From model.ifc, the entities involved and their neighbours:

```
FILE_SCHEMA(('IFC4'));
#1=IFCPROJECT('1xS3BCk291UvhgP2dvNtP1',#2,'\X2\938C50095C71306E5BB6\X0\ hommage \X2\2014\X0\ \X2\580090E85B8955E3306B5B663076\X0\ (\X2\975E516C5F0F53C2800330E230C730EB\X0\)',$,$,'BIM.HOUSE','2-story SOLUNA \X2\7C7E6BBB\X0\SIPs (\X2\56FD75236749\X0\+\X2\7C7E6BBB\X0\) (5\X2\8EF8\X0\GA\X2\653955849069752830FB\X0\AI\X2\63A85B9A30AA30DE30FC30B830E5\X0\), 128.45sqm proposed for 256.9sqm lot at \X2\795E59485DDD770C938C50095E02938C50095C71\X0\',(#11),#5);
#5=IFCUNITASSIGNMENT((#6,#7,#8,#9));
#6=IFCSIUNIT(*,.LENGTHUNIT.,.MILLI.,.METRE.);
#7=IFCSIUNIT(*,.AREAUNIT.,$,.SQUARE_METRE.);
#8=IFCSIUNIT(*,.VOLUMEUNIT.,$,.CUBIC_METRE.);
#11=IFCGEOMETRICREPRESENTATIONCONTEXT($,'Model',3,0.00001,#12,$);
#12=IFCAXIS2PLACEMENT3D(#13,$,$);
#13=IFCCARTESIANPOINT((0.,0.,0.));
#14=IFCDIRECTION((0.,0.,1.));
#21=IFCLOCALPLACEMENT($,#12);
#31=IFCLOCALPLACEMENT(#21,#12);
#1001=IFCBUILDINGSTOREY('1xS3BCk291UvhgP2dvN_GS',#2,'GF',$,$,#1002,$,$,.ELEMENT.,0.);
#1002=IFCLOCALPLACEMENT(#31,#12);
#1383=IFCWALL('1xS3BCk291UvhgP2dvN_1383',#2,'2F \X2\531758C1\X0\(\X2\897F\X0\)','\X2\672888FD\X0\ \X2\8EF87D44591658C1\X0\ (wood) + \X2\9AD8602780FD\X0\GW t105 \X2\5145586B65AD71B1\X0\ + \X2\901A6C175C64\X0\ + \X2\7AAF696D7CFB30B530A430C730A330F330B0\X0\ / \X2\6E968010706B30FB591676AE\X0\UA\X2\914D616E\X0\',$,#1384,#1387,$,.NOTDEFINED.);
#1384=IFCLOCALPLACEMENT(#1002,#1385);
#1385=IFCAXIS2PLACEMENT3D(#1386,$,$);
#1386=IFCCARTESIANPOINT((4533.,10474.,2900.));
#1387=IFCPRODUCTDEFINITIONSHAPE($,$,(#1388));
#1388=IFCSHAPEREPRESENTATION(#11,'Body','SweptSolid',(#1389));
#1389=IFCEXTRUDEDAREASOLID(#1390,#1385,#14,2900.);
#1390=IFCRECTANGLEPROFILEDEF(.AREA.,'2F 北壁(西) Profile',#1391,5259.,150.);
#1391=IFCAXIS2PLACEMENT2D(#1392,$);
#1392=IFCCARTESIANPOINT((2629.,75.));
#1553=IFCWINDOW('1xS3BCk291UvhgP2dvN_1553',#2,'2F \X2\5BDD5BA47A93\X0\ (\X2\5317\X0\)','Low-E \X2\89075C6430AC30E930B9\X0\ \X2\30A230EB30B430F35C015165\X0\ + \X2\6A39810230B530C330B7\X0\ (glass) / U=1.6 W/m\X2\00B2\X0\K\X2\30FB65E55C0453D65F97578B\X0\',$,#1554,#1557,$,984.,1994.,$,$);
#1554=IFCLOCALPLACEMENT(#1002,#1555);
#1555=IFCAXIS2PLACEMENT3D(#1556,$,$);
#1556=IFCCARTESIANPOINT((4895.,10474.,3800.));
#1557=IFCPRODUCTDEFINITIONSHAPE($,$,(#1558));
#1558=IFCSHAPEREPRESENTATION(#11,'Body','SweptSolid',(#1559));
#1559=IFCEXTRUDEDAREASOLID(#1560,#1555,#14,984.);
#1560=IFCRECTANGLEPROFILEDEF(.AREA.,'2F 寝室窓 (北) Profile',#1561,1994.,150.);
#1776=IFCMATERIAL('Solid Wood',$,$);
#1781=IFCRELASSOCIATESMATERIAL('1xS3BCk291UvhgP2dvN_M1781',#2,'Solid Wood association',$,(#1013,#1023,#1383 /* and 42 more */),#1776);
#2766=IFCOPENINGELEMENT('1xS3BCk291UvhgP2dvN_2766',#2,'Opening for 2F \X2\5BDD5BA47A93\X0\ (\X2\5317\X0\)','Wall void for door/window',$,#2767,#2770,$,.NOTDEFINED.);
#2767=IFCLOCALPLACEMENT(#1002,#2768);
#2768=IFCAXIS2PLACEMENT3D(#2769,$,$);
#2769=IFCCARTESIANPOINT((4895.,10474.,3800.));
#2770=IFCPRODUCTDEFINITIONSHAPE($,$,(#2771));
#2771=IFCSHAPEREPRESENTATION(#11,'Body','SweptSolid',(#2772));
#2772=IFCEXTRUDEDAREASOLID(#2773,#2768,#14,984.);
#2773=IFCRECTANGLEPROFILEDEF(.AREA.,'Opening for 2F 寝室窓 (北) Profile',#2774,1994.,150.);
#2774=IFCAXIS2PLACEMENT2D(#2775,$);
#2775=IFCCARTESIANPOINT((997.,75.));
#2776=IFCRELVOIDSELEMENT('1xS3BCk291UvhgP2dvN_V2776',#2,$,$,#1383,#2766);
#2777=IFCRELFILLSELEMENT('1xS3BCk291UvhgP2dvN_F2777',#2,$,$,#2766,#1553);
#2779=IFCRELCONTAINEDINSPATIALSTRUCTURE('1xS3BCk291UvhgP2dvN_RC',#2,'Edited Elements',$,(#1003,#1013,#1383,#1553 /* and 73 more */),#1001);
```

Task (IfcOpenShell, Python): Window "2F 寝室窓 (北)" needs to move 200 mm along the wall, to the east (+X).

```python
import ifcopenshell
import ifcopenshell.api.geometry
import ifcopenshell.util.placement

model = ifcopenshell.open("model.ifc")

window = model.by_guid("1xS3BCk291UvhgP2dvN_1553")
opening = window.FillsVoids[0].RelatingOpeningElement
wall = opening.VoidsElements[0].RelatingBuildingElement

wall_matrix = ifcopenshell.util.placement.get_local_placement(wall.ObjectPlacement)
shift = wall_matrix[:3, 0] * 200.0
before = ifcopenshell.util.placement.get_local_placement(window.ObjectPlacement)[:3, 3].copy()

# The window is not placed relative to its opening, so move both.
for product in (opening, window):
    matrix = ifcopenshell.util.placement.get_local_placement(product.ObjectPlacement)
    matrix[:3, 3] += shift
    ifcopenshell.api.geometry.edit_object_placement(model, product=product, matrix=matrix, is_si=False)

after = ifcopenshell.util.placement.get_local_placement(window.ObjectPlacement)[:3, 3]
print("window moved by", (after - before).round(3) + 0.0)

model.write("model-out.ifc")
```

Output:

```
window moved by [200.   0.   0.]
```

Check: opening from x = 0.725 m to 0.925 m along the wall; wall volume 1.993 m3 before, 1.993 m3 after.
